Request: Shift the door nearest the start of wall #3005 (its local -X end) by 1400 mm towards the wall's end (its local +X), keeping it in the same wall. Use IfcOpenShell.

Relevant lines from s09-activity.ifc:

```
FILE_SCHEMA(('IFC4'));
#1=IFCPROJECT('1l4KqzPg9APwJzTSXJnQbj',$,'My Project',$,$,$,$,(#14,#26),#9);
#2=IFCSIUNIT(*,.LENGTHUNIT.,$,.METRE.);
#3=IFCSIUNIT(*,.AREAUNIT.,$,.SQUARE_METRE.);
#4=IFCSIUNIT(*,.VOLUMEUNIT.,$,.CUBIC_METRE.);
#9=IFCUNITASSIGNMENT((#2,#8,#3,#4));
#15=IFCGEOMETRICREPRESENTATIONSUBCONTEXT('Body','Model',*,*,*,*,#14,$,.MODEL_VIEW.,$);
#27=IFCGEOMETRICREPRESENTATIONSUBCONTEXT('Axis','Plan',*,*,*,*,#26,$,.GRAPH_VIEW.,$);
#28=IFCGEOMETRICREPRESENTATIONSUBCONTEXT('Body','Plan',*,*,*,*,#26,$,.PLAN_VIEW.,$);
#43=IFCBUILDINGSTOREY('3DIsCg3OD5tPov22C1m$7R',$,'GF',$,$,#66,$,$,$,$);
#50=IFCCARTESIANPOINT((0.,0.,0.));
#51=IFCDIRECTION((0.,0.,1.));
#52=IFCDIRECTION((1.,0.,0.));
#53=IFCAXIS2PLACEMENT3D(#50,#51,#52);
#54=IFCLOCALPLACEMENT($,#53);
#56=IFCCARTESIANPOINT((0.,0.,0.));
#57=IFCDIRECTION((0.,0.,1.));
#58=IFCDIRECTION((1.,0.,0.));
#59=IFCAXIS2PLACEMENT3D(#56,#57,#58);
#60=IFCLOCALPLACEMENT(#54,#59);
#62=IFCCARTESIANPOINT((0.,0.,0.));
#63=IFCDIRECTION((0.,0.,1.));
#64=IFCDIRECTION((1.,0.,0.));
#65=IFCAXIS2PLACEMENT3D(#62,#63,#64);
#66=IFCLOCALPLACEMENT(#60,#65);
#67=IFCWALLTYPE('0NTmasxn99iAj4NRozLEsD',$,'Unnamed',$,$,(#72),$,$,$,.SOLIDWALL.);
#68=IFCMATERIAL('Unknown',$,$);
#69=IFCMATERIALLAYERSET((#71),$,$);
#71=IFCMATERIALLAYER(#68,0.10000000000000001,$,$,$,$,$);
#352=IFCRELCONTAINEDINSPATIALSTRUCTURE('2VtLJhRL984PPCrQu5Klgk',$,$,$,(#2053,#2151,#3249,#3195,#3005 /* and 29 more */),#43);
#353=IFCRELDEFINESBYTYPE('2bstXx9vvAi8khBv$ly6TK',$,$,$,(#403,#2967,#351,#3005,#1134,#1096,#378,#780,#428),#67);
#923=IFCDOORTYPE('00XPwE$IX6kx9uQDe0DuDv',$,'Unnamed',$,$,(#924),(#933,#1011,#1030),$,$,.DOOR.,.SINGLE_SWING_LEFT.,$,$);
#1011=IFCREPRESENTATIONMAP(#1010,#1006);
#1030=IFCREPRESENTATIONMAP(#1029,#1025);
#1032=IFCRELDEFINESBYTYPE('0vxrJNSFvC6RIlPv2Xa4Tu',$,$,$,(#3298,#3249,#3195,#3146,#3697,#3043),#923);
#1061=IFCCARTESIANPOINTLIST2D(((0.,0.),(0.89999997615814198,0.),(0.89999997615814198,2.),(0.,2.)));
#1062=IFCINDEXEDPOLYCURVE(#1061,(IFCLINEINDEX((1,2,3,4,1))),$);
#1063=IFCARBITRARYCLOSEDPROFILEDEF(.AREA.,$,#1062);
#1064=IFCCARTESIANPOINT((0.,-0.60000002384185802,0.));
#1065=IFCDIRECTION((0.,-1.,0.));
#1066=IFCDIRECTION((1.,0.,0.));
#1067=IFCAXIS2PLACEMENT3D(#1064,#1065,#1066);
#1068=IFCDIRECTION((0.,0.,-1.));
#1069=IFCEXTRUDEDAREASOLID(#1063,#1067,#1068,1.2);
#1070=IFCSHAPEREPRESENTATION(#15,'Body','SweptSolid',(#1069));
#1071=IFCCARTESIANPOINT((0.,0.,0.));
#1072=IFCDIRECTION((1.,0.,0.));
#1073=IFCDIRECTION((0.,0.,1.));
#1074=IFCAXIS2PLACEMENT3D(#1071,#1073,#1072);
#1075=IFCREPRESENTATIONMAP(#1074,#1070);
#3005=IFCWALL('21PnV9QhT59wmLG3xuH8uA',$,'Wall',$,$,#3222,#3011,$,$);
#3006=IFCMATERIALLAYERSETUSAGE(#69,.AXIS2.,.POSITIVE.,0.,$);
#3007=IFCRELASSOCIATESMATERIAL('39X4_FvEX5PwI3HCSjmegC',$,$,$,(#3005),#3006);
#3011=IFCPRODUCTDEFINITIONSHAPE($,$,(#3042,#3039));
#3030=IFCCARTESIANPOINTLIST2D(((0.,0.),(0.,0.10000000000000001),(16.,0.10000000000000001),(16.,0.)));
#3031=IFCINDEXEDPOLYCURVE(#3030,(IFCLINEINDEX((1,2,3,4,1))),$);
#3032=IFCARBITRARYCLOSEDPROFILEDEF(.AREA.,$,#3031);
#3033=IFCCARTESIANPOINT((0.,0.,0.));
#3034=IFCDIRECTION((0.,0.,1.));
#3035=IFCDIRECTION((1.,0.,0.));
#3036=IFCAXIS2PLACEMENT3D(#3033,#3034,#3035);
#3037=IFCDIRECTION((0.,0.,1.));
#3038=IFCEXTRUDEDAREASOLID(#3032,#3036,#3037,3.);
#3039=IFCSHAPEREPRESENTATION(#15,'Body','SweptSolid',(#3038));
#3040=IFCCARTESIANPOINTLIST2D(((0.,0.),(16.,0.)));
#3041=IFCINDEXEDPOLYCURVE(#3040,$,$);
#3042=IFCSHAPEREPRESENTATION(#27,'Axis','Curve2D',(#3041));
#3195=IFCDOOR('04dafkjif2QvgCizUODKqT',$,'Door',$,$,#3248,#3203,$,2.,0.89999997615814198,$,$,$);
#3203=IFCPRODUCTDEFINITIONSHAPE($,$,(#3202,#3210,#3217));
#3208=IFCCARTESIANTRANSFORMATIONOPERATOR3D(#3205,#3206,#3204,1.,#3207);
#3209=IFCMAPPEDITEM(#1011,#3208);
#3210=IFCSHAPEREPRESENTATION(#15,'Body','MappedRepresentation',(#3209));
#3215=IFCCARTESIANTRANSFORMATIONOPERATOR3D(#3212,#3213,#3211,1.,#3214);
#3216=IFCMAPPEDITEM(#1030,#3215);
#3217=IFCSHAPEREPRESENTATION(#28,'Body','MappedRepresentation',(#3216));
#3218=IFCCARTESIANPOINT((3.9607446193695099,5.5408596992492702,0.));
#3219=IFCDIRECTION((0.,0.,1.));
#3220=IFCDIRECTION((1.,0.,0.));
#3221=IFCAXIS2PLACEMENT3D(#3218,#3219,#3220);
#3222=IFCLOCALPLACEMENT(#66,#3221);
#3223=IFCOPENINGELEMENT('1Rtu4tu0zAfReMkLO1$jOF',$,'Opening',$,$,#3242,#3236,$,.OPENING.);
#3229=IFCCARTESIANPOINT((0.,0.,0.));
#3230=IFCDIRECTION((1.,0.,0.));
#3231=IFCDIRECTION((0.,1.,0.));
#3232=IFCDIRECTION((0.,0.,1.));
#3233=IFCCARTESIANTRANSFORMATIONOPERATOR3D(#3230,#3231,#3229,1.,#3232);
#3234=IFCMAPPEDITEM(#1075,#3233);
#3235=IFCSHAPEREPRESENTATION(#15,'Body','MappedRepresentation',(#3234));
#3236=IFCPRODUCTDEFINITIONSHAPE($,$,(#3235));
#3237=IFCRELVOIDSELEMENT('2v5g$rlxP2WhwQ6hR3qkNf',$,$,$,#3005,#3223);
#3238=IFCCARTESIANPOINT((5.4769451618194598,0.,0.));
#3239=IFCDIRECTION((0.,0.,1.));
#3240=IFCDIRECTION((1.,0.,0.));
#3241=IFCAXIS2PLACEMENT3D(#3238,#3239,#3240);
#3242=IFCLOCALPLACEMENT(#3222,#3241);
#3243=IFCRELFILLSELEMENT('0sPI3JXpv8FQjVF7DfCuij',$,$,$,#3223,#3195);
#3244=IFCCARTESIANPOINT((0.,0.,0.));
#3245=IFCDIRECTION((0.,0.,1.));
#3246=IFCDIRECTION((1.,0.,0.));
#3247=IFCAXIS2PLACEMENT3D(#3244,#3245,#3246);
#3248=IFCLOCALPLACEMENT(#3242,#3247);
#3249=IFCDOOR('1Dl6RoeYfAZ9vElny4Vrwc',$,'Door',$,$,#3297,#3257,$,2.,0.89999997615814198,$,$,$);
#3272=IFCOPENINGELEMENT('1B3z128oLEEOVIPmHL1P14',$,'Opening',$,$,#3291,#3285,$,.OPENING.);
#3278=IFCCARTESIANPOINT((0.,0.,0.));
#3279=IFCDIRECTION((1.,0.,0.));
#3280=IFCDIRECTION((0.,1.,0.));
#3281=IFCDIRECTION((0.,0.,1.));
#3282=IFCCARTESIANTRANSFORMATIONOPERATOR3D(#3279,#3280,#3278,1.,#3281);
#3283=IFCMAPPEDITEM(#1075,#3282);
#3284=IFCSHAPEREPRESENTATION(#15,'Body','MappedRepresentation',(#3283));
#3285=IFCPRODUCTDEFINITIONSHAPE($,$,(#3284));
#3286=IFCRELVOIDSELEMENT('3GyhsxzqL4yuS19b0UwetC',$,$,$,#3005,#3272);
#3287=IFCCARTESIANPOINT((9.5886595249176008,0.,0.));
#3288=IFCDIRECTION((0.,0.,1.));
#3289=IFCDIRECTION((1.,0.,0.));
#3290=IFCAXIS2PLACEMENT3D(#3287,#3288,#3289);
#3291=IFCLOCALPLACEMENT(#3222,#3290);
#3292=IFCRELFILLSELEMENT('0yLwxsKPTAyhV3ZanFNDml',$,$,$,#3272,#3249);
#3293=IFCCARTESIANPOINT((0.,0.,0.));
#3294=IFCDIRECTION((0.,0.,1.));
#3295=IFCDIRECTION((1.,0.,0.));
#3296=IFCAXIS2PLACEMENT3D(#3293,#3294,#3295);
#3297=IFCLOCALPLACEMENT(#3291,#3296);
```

```python
import ifcopenshell
import ifcopenshell.api.geometry
import ifcopenshell.util.placement

model = ifcopenshell.open("s09-activity.ifc")

door = model.by_id(3195)
opening = door.FillsVoids[0].RelatingOpeningElement
wall = opening.VoidsElements[0].RelatingBuildingElement

wall_matrix = ifcopenshell.util.placement.get_local_placement(wall.ObjectPlacement)
shift = wall_matrix[:3, 0] * 1.4
before = ifcopenshell.util.placement.get_local_placement(door.ObjectPlacement)[:3, 3].copy()

# The door is placed relative to its opening, so it follows when the opening moves.
matrix = ifcopenshell.util.placement.get_local_placement(opening.ObjectPlacement)
matrix[:3, 3] += shift
ifcopenshell.api.geometry.edit_object_placement(
    model, product=opening, matrix=matrix, is_si=False, should_transform_children=True
)

after = ifcopenshell.util.placement.get_local_placement(door.ObjectPlacement)[:3, 3]
print("door moved by", (after - before).round(3) + 0.0)

model.write("s09-activity-out.ifc")
```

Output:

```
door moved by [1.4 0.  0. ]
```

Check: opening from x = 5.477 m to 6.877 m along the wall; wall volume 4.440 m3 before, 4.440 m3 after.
